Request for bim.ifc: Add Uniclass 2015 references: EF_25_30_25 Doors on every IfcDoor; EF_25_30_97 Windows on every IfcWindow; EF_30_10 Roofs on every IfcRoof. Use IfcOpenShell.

First a look at what the model holds.

```python
import ifcopenshell

model = ifcopenshell.open("bim.ifc")
print(model.schema)
print("classifications:", [c.Name for c in model.by_type("IfcClassification")])
for ifc_class in ("IfcDoor", "IfcRoof", "IfcStair", "IfcWall", "IfcWindow"):
    print(ifc_class, len(model.by_type(ifc_class)))
```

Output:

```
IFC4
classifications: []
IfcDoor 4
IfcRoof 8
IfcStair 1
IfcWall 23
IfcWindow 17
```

```python
import ifcopenshell
import ifcopenshell.api.classification

model = ifcopenshell.open("bim.ifc")

system = ifcopenshell.api.classification.add_classification(model, classification="Uniclass 2015")

codes = {
    "IfcDoor": ("EF_25_30_25", "Doors"),
    "IfcWindow": ("EF_25_30_97", "Windows"),
    "IfcRoof": ("EF_30_10", "Roofs"),
}
for ifc_class, (code, name) in codes.items():
    products = model.by_type(ifc_class)
    ifcopenshell.api.classification.add_reference(
        model, products=products, classification=system, identification=code, name=name
    )
    print(code, len(products))

model.write("bim_rev.ifc")
```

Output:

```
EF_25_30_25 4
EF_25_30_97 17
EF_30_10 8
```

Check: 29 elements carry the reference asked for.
